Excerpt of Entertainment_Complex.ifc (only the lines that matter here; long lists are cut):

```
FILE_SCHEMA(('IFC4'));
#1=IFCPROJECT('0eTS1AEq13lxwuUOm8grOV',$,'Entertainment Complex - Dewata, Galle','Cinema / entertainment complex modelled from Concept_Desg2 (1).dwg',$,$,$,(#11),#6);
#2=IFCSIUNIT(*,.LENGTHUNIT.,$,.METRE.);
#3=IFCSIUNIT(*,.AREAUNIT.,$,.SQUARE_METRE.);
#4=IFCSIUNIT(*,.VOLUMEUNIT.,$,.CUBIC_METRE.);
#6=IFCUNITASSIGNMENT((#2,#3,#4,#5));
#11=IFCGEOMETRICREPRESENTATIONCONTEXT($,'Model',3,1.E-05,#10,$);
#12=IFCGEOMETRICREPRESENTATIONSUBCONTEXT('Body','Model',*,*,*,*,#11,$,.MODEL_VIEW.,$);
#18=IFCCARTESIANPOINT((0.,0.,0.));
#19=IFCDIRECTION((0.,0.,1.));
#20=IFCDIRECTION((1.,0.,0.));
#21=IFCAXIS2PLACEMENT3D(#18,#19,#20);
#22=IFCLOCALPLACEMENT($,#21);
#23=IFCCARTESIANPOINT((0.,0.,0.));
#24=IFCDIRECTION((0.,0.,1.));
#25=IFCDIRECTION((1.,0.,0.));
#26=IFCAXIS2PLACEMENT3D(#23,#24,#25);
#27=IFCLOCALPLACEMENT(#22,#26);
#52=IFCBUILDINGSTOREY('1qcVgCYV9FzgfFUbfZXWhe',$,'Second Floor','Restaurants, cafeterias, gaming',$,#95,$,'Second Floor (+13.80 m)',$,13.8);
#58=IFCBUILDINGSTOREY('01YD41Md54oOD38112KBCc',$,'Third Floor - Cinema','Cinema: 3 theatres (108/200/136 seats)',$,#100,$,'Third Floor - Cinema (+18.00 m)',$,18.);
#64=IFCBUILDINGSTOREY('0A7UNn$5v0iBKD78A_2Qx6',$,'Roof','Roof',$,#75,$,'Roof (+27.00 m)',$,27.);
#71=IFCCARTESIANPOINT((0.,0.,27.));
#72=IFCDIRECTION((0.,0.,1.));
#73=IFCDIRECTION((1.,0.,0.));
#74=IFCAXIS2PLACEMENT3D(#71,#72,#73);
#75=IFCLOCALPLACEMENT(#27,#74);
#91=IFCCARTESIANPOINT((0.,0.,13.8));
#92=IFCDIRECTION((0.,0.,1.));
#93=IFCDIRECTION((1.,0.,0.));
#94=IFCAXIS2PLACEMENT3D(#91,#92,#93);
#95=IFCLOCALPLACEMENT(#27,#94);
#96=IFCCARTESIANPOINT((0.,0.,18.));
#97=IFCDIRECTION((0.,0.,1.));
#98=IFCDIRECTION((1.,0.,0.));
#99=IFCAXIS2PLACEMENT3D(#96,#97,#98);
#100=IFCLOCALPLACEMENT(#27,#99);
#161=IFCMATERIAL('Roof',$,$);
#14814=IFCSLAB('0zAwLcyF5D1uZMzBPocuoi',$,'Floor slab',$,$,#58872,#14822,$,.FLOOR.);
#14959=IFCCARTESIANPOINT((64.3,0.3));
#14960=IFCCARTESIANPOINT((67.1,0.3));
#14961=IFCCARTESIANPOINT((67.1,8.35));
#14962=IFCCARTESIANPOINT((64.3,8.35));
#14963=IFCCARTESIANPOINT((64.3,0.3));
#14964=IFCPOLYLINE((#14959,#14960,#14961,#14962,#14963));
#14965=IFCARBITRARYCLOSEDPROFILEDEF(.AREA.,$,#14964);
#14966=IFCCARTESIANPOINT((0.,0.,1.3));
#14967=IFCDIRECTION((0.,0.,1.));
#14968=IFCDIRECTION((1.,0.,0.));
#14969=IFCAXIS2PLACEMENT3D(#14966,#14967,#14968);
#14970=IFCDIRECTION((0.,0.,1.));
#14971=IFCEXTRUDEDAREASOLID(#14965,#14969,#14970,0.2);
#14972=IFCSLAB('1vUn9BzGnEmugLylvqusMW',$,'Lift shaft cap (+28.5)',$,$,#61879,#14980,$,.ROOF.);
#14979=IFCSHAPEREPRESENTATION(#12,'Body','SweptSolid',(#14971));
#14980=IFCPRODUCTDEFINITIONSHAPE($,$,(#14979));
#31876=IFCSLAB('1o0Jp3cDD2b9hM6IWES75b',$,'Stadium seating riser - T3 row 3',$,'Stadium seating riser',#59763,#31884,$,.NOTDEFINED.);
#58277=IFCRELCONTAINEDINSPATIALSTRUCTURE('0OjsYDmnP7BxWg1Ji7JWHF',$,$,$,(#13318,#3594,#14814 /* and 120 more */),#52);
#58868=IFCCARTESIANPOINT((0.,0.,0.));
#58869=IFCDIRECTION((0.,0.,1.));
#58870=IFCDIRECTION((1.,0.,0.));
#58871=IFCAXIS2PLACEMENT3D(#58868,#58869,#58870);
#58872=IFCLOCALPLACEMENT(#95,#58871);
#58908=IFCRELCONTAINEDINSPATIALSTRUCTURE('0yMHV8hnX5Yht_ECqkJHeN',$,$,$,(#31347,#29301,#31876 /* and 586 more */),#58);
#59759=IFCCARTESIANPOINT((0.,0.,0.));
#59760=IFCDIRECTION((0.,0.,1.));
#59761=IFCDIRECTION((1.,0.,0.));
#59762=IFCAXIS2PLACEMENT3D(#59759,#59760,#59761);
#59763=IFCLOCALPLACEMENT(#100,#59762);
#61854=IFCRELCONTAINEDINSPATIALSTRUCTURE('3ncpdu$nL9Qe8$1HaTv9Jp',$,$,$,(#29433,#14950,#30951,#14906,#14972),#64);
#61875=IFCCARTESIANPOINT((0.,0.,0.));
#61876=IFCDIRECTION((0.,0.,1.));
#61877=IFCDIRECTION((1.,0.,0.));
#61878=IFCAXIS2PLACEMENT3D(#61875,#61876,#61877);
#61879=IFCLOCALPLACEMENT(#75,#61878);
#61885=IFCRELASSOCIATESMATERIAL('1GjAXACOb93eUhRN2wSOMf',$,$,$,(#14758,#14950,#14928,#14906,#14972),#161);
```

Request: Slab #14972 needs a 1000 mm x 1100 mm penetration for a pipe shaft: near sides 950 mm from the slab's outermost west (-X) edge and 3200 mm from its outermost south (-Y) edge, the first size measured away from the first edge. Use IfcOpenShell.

```python
import numpy as np
import ifcopenshell
import ifcopenshell.api.feature
import ifcopenshell.api.geometry
import ifcopenshell.api.root
import ifcopenshell.geom
import ifcopenshell.util.placement
import ifcopenshell.util.representation
import ifcopenshell.util.shape
import ifcopenshell.util.unit

model = ifcopenshell.open("Entertainment_Complex.ifc")
unit_scale = ifcopenshell.util.unit.calculate_unit_scale(model)
settings = ifcopenshell.geom.settings()


def volume(element):
    """Net volume in cubic metres, openings subtracted."""
    shape = ifcopenshell.geom.create_shape(settings, element)
    return ifcopenshell.util.shape.get_volume(shape.geometry)


slab = model.by_id(14972)
before = volume(slab)

# Extent in the slab's own axes, in metres. The edges named are its -X and -Y sides.
slab_shape = ifcopenshell.geom.create_shape(settings, slab)
vertices = ifcopenshell.util.shape.get_vertices(slab_shape.geometry)
x_min, y_min, bottom = vertices.min(axis=0)
top = vertices[:, 2].max()

opening = ifcopenshell.api.root.create_entity(model, ifc_class="IfcOpeningElement", name="Pipe shaft opening", predefined_type="OPENING")
context = ifcopenshell.util.representation.get_context(model, "Model", "Body", "MODEL_VIEW")
width, depth = 1, 1.1
outline = [(0.0, 0.0), (width, 0.0), (width, depth), (0.0, depth), (0.0, 0.0)]
# Overshoot both faces by 50 mm so the cut is clean.
shape = ifcopenshell.api.geometry.add_slab_representation(
    model, context=context, depth=top - bottom + 0.1, polyline=outline
)
ifcopenshell.api.geometry.assign_representation(model, product=opening, representation=shape)

matrix = ifcopenshell.util.placement.get_local_placement(slab.ObjectPlacement)
matrix[:, 3] = matrix @ np.append(np.array([x_min + 0.95, y_min + 3.2, bottom - 0.05]) / unit_scale, 1.0)
ifcopenshell.api.geometry.edit_object_placement(model, product=opening, matrix=matrix, is_si=False)
ifcopenshell.api.feature.add_feature(model, feature=opening, element=slab)

after = volume(slab)

print(f"slab volume {before:.3f} -> {after:.3f} m3")

model.write("Entertainment_Complex-out.ifc")
```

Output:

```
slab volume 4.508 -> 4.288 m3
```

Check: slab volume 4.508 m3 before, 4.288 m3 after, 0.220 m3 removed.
